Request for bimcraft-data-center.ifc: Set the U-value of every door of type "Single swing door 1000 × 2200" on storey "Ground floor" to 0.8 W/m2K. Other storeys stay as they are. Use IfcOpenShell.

First a look at what the model holds.

```python
import ifcopenshell
import ifcopenshell.util.element

model = ifcopenshell.open("bimcraft-data-center.ifc")
print(model.schema)
storey = next(s for s in model.by_type("IfcBuildingStorey") if s.Name == "Ground floor")
doors = [e for e in ifcopenshell.util.element.get_decomposition(storey) if e.is_a("IfcDoor")]
seen = {}
for e in doors:
    element_type = ifcopenshell.util.element.get_type(e)
    key = (element_type.Name if element_type != e and element_type else None, ifcopenshell.util.element.get_pset(e, "Pset_DoorCommon", "ThermalTransmittance"))
    seen[key] = seen.get(key, 0) + 1
for (name, value), count in sorted(seen.items(), key=str):
    print(count, "x", name, "|", value)
```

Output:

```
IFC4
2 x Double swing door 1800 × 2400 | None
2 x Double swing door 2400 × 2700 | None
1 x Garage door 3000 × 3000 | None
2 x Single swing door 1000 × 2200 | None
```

```python
import ifcopenshell
import ifcopenshell.api.pset
import ifcopenshell.util.element

model = ifcopenshell.open("bimcraft-data-center.ifc")

storey = next(s for s in model.by_type("IfcBuildingStorey") if s.Name == "Ground floor")
doors = [e for e in ifcopenshell.util.element.get_decomposition(storey) if e.is_a("IfcDoor")]

count = 0
for e in doors:
    element_type = ifcopenshell.util.element.get_type(e)
    if element_type in (None, e) or element_type.Name != "Single swing door 1000 × 2200":
        continue
    # add_pset returns the element's existing set when there is one.
    pset = ifcopenshell.api.pset.add_pset(model, product=e, name="Pset_DoorCommon")
    ifcopenshell.api.pset.edit_pset(model, pset=pset, properties={"ThermalTransmittance": 0.8})
    count += 1

print(count, "doors updated")

model.write("bimcraft-data-center_v2.ifc")
```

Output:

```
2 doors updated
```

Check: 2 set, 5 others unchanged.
